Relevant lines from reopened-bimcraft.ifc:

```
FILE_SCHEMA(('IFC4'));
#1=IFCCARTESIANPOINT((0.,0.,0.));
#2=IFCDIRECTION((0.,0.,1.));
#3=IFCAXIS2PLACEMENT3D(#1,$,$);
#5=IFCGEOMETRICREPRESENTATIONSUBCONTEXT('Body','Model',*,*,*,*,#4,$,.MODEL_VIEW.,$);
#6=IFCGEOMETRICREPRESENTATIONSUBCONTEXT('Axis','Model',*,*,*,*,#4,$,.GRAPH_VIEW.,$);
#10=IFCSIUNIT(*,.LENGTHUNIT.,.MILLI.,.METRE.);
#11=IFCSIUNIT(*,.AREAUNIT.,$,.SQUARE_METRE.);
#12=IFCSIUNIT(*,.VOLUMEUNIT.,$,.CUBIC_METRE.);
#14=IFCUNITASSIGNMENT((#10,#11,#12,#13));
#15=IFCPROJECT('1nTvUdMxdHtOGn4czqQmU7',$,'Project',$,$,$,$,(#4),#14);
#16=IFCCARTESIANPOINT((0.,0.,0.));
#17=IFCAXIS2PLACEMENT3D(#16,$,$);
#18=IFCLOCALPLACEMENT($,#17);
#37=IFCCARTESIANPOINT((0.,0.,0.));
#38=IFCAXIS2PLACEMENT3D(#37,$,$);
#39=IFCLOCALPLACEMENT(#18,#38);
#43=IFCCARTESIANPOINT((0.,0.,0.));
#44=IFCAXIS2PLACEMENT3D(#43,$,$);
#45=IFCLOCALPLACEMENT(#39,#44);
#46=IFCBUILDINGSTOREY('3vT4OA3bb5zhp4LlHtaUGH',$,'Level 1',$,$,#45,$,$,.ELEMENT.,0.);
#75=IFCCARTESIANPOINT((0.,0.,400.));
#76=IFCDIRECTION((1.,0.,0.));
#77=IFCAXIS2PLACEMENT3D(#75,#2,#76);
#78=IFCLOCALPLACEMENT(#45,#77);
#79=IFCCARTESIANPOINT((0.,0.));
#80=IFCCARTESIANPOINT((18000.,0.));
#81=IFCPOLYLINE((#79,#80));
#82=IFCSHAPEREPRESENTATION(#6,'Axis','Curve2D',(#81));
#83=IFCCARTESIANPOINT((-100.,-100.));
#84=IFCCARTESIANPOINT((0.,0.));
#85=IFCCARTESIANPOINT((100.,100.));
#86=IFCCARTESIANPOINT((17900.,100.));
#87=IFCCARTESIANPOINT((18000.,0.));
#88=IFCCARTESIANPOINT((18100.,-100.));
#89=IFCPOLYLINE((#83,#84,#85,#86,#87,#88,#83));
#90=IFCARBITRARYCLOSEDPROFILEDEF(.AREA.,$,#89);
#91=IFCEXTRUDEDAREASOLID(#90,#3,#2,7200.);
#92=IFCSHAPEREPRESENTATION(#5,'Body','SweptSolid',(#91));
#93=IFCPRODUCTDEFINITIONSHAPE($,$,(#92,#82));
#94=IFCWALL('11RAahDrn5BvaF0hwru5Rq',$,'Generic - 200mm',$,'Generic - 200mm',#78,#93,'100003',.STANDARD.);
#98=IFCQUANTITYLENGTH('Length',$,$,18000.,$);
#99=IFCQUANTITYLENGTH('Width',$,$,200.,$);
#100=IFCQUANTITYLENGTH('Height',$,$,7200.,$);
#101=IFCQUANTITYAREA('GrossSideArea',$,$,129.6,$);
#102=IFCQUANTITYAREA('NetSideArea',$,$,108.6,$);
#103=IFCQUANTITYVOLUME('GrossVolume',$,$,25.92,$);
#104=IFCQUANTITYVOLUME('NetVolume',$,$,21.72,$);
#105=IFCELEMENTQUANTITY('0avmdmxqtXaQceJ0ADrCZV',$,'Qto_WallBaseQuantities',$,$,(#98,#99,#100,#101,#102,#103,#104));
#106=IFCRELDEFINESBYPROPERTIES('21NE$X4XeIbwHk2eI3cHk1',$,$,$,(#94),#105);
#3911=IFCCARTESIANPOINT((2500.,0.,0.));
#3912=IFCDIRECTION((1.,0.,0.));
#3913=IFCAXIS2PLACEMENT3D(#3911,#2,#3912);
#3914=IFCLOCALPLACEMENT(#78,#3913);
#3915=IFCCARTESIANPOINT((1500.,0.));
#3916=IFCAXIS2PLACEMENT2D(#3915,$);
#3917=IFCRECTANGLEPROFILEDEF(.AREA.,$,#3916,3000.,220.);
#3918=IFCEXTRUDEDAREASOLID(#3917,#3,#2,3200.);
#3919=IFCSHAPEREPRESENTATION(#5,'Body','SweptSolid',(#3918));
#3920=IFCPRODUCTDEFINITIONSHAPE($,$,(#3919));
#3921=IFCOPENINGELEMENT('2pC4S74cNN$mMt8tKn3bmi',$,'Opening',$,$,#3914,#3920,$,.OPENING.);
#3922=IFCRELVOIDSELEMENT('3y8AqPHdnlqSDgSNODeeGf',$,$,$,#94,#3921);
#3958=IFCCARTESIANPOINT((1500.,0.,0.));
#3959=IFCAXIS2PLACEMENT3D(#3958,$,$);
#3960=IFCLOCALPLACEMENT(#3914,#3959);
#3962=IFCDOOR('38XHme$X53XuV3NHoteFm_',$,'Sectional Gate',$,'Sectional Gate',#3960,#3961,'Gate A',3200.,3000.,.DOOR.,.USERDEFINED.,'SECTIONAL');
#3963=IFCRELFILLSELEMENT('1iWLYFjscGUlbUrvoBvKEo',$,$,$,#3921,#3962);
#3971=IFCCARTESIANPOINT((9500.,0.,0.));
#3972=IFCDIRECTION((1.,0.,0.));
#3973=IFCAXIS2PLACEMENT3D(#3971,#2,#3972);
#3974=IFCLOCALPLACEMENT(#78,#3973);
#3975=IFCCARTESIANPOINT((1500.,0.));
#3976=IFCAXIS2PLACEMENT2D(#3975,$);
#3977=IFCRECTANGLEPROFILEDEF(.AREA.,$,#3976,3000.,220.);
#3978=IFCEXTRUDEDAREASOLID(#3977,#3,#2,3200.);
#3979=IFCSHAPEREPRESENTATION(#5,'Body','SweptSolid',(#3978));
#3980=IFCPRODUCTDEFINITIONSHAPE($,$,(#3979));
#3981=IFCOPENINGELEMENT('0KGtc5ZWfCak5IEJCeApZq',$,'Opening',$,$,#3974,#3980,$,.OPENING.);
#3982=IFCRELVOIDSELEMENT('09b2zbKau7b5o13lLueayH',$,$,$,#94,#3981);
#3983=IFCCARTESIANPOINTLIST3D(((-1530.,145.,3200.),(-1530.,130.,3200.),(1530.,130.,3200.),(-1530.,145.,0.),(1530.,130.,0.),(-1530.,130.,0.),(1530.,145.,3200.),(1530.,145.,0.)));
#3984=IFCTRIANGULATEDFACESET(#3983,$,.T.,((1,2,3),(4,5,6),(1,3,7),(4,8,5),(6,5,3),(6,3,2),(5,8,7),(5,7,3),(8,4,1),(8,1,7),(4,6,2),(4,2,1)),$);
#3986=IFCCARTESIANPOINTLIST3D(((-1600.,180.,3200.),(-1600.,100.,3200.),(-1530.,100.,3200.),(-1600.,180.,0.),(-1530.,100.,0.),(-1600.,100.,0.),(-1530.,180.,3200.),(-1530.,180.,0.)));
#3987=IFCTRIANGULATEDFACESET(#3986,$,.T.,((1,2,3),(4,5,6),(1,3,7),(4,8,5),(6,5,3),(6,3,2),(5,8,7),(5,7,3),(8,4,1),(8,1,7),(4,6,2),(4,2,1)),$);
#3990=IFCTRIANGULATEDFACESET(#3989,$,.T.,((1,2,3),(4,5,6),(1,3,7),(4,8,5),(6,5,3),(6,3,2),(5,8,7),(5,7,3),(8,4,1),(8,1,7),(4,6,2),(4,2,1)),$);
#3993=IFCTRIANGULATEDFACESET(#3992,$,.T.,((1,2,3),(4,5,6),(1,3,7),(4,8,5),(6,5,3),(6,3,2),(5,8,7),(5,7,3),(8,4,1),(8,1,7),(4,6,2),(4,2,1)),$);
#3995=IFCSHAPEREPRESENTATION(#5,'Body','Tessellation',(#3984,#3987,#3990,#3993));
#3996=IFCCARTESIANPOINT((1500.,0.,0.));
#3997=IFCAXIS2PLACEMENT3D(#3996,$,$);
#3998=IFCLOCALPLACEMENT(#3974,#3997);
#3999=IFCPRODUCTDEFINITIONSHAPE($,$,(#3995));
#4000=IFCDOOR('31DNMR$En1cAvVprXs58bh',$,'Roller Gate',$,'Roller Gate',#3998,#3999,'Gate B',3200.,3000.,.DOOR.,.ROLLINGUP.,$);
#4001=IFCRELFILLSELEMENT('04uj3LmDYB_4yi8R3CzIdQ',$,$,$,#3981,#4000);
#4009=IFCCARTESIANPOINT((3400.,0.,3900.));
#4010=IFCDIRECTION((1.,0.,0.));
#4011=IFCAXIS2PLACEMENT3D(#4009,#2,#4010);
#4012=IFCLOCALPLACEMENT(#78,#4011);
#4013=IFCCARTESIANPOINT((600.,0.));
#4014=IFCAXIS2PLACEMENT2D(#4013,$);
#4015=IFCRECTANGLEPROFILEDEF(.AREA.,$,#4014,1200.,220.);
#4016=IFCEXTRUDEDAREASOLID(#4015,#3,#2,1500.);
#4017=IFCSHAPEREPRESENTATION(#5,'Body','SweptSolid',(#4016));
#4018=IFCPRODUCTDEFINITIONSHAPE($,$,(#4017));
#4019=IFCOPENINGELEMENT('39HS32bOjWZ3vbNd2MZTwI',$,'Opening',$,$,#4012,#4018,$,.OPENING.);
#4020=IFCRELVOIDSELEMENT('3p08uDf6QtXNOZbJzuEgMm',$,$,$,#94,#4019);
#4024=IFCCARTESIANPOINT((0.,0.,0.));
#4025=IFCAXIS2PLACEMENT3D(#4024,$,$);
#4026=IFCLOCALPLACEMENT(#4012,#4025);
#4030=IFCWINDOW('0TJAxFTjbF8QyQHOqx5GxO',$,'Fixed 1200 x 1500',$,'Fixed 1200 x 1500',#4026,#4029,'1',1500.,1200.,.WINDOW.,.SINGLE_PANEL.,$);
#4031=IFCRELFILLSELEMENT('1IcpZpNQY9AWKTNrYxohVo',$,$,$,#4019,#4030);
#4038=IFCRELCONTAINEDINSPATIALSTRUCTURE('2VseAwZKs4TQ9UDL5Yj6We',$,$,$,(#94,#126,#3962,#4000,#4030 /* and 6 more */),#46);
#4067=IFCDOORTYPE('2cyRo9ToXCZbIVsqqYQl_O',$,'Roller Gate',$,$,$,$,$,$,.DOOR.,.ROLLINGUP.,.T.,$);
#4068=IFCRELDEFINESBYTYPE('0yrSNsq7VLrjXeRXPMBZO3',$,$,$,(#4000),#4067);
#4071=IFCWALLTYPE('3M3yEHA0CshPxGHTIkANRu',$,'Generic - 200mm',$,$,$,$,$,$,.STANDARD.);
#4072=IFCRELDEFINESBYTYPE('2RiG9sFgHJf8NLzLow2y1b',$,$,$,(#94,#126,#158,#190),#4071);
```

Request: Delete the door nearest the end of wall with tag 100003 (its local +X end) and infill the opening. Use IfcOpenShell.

```python
import ifcopenshell
import ifcopenshell.api.feature
import ifcopenshell.api.pset
import ifcopenshell.api.root
import ifcopenshell.geom
import ifcopenshell.util.element
import ifcopenshell.util.shape
import ifcopenshell.util.unit

model = ifcopenshell.open("reopened-bimcraft.ifc")
area_scale = ifcopenshell.util.unit.calculate_unit_scale(model, "AREAUNIT")
volume_scale = ifcopenshell.util.unit.calculate_unit_scale(model, "VOLUMEUNIT")
settings = ifcopenshell.geom.settings()


def volume(element):
    """Net volume in cubic metres, openings subtracted."""
    shape = ifcopenshell.geom.create_shape(settings, element)
    return ifcopenshell.util.shape.get_volume(shape.geometry)


door = model.by_guid("31DNMR$En1cAvVprXs58bh")
opening = door.FillsVoids[0].RelatingOpeningElement
wall = opening.VoidsElements[0].RelatingBuildingElement
before = volume(wall)

ifcopenshell.api.root.remove_product(model, product=door)
ifcopenshell.api.feature.remove_feature(model, feature=opening)

after = volume(wall)
thickness = 0.2  # wall thickness in metres

# Update the wall's stored quantities.
qto = model.by_id(ifcopenshell.util.element.get_pset(wall, "Qto_WallBaseQuantities", should_inherit=False)["id"])
ifcopenshell.api.pset.edit_qto(model, qto=qto, properties={
    "NetSideArea": after / thickness / area_scale,
    "NetVolume": after / volume_scale,
})

print(f"wall volume {before:.3f} -> {after:.3f} m3")

model.write("reopened-bimcraft_rev.ifc")
```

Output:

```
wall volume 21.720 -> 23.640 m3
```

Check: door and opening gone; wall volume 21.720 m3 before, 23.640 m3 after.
